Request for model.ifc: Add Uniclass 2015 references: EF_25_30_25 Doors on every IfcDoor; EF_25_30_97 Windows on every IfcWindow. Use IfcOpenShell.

First a look at what the model holds.

```python
import ifcopenshell

model = ifcopenshell.open("model.ifc")
print(model.schema)
print("classifications:", [c.Name for c in model.by_type("IfcClassification")])
for ifc_class in ("IfcDoor", "IfcRoof", "IfcStair", "IfcWall", "IfcWindow"):
    print(ifc_class, len(model.by_type(ifc_class)))
```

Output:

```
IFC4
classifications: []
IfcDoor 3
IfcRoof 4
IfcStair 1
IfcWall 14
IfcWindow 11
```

```python
import ifcopenshell
import ifcopenshell.api.classification

model = ifcopenshell.open("model.ifc")

system = ifcopenshell.api.classification.add_classification(model, classification="Uniclass 2015")

codes = {
    "IfcDoor": ("EF_25_30_25", "Doors"),
    "IfcWindow": ("EF_25_30_97", "Windows"),
}
for ifc_class, (code, name) in codes.items():
    products = model.by_type(ifc_class)
    ifcopenshell.api.classification.add_reference(
        model, products=products, classification=system, identification=code, name=name
    )
    print(code, len(products))

model.write("model_rev.ifc")
```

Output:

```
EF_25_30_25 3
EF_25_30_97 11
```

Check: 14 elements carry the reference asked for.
